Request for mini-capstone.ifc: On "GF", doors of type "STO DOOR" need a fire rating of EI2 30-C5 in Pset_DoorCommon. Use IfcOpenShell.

First a look at what the model holds.

```python
import ifcopenshell
import ifcopenshell.util.element

model = ifcopenshell.open("mini-capstone.ifc")
print(model.schema)
storey = next(s for s in model.by_type("IfcBuildingStorey") if s.Name == "GF")
doors = [e for e in ifcopenshell.util.element.get_decomposition(storey) if e.is_a("IfcDoor")]
seen = {}
for e in doors:
    element_type = ifcopenshell.util.element.get_type(e)
    key = (element_type.Name if element_type != e and element_type else None, ifcopenshell.util.element.get_pset(e, "Pset_DoorCommon", "FireRating"))
    seen[key] = seen.get(key, 0) + 1
for (name, value), count in sorted(seen.items(), key=str):
    print(count, "x", name, "|", value)
```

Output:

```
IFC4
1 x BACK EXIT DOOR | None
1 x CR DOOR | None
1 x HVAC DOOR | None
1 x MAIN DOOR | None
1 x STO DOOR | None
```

```python
import ifcopenshell
import ifcopenshell.api.pset
import ifcopenshell.util.element

model = ifcopenshell.open("mini-capstone.ifc")

storey = next(s for s in model.by_type("IfcBuildingStorey") if s.Name == "GF")
doors = [e for e in ifcopenshell.util.element.get_decomposition(storey) if e.is_a("IfcDoor")]

count = 0
for e in doors:
    element_type = ifcopenshell.util.element.get_type(e)
    if element_type in (None, e) or element_type.Name != "STO DOOR":
        continue
    # add_pset returns the element's existing set when there is one.
    pset = ifcopenshell.api.pset.add_pset(model, product=e, name="Pset_DoorCommon")
    ifcopenshell.api.pset.edit_pset(model, pset=pset, properties={"FireRating": "EI2 30-C5"})
    count += 1

print(count, "doors updated")

model.write("mini-capstone_edited.ifc")
```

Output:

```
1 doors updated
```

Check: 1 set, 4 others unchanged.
